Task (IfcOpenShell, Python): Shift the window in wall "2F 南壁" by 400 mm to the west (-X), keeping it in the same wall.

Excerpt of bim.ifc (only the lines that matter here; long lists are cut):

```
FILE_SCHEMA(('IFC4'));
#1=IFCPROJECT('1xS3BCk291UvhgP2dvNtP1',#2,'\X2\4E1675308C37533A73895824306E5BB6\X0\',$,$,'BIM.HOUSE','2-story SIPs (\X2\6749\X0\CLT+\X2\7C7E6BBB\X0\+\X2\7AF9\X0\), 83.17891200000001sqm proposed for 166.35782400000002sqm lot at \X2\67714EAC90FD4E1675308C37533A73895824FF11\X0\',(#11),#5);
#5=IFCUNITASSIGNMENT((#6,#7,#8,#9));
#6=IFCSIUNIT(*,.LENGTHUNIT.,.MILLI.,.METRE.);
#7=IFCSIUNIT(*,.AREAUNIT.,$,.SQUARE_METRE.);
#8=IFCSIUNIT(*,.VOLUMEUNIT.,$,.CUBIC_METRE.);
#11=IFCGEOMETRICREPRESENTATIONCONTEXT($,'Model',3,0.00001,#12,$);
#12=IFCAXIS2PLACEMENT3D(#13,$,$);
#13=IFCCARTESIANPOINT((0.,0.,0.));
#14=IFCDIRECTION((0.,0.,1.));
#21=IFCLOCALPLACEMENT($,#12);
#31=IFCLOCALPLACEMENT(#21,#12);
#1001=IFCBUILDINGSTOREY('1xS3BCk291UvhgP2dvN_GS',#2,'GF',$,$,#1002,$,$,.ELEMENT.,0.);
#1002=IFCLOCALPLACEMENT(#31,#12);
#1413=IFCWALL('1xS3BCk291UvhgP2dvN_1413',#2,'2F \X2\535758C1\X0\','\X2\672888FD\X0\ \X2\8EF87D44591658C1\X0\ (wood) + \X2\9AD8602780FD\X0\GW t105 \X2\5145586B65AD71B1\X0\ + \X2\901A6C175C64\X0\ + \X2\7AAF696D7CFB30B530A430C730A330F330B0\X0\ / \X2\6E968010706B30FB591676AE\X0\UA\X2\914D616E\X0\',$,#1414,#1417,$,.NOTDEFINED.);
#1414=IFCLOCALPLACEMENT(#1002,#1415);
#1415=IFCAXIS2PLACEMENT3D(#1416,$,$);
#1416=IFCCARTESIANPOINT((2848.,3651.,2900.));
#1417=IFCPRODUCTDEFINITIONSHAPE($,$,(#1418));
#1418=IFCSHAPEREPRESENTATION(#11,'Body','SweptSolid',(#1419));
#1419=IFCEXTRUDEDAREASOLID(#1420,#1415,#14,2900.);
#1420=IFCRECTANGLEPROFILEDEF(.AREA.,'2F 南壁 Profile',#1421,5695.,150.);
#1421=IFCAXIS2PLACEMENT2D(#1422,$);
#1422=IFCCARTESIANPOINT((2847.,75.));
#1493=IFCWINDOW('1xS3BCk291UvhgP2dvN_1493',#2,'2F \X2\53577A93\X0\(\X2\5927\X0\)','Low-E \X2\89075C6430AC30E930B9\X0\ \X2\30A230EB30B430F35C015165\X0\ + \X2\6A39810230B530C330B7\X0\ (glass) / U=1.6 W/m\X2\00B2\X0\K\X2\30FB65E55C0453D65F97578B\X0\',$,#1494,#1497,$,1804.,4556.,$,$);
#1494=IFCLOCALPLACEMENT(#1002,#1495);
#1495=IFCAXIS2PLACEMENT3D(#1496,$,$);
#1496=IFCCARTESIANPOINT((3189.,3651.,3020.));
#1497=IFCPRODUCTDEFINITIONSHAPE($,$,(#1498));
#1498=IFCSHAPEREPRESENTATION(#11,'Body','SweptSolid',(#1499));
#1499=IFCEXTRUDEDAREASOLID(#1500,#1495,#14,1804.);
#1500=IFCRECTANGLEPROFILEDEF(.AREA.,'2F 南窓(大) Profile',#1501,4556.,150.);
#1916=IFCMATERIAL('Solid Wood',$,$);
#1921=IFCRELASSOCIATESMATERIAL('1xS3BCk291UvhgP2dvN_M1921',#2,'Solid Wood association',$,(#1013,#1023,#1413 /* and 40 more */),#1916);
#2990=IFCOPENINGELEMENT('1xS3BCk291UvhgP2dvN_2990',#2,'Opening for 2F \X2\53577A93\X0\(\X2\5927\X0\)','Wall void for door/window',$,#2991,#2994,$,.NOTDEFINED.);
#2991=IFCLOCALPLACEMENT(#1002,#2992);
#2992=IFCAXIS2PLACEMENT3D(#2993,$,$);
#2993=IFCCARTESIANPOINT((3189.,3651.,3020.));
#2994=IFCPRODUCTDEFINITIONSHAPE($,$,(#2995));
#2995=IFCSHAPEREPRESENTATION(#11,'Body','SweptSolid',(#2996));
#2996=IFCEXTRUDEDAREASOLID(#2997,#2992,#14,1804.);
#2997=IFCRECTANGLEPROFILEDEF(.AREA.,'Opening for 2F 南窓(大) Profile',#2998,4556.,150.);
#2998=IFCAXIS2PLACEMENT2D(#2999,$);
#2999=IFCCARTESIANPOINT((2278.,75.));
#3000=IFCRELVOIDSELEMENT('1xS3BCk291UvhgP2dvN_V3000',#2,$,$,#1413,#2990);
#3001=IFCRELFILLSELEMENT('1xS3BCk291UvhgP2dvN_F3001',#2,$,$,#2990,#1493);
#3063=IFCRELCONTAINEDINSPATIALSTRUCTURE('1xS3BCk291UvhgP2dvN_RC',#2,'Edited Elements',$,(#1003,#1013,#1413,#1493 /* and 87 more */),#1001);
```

```python
import ifcopenshell
import ifcopenshell.api.geometry
import ifcopenshell.util.placement
import ifcopenshell.util.unit

model = ifcopenshell.open("bim.ifc")
unit_scale = ifcopenshell.util.unit.calculate_unit_scale(model)

window = model.by_guid("1xS3BCk291UvhgP2dvN_1493")
opening = window.FillsVoids[0].RelatingOpeningElement
wall = opening.VoidsElements[0].RelatingBuildingElement

wall_matrix = ifcopenshell.util.placement.get_local_placement(wall.ObjectPlacement)
shift = wall_matrix[:3, 0] * -0.4 / unit_scale
before = ifcopenshell.util.placement.get_local_placement(window.ObjectPlacement)[:3, 3].copy()

# The window is not placed relative to its opening, so move both.
for product in (opening, window):
    matrix = ifcopenshell.util.placement.get_local_placement(product.ObjectPlacement)
    matrix[:3, 3] += shift
    ifcopenshell.api.geometry.edit_object_placement(model, product=product, matrix=matrix, is_si=False)

after = ifcopenshell.util.placement.get_local_placement(window.ObjectPlacement)[:3, 3]
print("window moved by", (after - before).round(3) + 0.0)

model.write("bim_v2.ifc")
```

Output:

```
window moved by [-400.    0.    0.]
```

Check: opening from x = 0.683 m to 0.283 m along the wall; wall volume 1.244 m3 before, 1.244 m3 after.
